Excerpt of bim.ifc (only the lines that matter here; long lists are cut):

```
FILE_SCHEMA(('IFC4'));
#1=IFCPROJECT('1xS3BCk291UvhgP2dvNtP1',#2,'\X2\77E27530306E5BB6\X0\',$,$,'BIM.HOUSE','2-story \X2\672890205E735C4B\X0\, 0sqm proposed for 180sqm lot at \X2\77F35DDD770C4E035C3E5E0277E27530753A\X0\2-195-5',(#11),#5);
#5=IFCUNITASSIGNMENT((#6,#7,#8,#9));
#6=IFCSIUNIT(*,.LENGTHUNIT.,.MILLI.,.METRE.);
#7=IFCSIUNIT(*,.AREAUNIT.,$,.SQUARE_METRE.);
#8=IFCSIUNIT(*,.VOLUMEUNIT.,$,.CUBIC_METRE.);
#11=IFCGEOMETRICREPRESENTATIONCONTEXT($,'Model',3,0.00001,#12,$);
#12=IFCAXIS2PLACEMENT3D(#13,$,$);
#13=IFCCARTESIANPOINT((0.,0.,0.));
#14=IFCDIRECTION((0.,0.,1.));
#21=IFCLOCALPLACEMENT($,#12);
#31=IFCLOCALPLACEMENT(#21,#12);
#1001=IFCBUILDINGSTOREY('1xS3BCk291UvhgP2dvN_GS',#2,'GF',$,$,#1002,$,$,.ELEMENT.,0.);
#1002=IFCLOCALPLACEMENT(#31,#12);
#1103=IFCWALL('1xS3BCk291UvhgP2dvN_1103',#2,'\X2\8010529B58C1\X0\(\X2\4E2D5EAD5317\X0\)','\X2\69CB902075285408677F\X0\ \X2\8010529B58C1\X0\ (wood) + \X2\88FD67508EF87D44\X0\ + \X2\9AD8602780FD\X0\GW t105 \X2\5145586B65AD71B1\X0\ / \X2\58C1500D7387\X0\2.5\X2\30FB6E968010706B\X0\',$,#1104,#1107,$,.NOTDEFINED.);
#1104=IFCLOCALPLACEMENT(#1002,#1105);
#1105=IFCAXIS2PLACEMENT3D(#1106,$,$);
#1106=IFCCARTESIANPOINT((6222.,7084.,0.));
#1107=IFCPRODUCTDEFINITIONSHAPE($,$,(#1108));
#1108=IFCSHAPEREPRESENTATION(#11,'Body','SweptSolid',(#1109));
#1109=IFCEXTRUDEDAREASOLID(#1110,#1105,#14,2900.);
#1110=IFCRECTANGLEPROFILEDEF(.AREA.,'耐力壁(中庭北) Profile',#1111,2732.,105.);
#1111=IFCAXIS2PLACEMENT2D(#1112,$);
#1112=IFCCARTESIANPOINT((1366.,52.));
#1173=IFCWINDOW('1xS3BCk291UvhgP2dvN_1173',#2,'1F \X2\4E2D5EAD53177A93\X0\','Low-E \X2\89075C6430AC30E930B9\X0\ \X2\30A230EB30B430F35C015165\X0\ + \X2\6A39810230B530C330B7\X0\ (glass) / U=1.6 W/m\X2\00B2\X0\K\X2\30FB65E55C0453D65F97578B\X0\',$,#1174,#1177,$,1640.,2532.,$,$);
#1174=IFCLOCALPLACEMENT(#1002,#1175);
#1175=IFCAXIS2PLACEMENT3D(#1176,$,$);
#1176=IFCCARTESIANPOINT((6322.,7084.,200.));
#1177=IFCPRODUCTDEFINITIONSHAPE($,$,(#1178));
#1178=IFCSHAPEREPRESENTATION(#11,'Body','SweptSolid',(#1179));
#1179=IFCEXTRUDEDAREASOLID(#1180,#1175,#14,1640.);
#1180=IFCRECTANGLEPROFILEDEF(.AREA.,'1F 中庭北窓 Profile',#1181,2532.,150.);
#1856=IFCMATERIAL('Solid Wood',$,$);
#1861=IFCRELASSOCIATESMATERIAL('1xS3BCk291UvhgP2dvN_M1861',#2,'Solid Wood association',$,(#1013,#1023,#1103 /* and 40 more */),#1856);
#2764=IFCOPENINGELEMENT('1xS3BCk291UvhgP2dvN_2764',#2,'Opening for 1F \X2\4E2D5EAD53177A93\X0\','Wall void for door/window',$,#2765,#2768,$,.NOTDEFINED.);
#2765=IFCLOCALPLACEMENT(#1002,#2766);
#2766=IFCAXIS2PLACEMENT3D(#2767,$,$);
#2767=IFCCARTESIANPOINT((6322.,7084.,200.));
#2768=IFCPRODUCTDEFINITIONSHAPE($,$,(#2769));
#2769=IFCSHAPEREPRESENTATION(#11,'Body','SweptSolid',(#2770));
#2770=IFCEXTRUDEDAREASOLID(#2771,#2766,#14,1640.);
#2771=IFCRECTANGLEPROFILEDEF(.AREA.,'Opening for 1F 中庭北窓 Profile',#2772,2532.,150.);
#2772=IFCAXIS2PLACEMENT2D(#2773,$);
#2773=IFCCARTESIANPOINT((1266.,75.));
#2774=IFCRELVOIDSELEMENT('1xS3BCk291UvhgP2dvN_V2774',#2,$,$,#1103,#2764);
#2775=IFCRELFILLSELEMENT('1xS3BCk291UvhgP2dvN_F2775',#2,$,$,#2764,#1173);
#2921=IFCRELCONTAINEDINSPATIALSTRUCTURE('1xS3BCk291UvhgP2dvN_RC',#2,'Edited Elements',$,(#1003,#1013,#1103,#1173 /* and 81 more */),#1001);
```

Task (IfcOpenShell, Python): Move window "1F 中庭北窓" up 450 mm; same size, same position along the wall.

```python
import numpy as np
import ifcopenshell
import ifcopenshell.api.geometry
import ifcopenshell.util.placement
import ifcopenshell.util.unit

model = ifcopenshell.open("bim.ifc")
unit_scale = ifcopenshell.util.unit.calculate_unit_scale(model)

window = model.by_guid("1xS3BCk291UvhgP2dvN_1173")
opening = window.FillsVoids[0].RelatingOpeningElement
dz = 0.45 / unit_scale

shift = np.array([0.0, 0.0, dz])
# The window is not placed relative to its opening, so move both.
for product in (opening, window):
    matrix = ifcopenshell.util.placement.get_local_placement(product.ObjectPlacement)
    matrix[:3, 3] += shift
    ifcopenshell.api.geometry.edit_object_placement(model, product=product, matrix=matrix, is_si=False)

print(f"moved by {dz * unit_scale:+.3f} m")

model.write("bim_v2.ifc")
```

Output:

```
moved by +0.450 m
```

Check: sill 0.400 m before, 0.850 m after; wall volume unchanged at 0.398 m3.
